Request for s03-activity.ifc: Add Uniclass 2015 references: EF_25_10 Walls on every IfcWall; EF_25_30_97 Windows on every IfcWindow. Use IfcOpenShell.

First a look at what the model holds.

```python
import ifcopenshell

model = ifcopenshell.open("s03-activity.ifc")
print(model.schema)
print("classifications:", [c.Name for c in model.by_type("IfcClassification")])
for ifc_class in ("IfcDoor", "IfcRoof", "IfcStair", "IfcWall", "IfcWindow"):
    print(ifc_class, len(model.by_type(ifc_class)))
```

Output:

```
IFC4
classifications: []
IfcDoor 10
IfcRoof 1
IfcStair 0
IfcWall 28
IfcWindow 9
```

```python
import ifcopenshell
import ifcopenshell.api.classification

model = ifcopenshell.open("s03-activity.ifc")

system = ifcopenshell.api.classification.add_classification(model, classification="Uniclass 2015")

codes = {
    "IfcWall": ("EF_25_10", "Walls"),
    "IfcWindow": ("EF_25_30_97", "Windows"),
}
for ifc_class, (code, name) in codes.items():
    products = model.by_type(ifc_class)
    ifcopenshell.api.classification.add_reference(
        model, products=products, classification=system, identification=code, name=name
    )
    print(code, len(products))

model.write("s03-activity_rev.ifc")
```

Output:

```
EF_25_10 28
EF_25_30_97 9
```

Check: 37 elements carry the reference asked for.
